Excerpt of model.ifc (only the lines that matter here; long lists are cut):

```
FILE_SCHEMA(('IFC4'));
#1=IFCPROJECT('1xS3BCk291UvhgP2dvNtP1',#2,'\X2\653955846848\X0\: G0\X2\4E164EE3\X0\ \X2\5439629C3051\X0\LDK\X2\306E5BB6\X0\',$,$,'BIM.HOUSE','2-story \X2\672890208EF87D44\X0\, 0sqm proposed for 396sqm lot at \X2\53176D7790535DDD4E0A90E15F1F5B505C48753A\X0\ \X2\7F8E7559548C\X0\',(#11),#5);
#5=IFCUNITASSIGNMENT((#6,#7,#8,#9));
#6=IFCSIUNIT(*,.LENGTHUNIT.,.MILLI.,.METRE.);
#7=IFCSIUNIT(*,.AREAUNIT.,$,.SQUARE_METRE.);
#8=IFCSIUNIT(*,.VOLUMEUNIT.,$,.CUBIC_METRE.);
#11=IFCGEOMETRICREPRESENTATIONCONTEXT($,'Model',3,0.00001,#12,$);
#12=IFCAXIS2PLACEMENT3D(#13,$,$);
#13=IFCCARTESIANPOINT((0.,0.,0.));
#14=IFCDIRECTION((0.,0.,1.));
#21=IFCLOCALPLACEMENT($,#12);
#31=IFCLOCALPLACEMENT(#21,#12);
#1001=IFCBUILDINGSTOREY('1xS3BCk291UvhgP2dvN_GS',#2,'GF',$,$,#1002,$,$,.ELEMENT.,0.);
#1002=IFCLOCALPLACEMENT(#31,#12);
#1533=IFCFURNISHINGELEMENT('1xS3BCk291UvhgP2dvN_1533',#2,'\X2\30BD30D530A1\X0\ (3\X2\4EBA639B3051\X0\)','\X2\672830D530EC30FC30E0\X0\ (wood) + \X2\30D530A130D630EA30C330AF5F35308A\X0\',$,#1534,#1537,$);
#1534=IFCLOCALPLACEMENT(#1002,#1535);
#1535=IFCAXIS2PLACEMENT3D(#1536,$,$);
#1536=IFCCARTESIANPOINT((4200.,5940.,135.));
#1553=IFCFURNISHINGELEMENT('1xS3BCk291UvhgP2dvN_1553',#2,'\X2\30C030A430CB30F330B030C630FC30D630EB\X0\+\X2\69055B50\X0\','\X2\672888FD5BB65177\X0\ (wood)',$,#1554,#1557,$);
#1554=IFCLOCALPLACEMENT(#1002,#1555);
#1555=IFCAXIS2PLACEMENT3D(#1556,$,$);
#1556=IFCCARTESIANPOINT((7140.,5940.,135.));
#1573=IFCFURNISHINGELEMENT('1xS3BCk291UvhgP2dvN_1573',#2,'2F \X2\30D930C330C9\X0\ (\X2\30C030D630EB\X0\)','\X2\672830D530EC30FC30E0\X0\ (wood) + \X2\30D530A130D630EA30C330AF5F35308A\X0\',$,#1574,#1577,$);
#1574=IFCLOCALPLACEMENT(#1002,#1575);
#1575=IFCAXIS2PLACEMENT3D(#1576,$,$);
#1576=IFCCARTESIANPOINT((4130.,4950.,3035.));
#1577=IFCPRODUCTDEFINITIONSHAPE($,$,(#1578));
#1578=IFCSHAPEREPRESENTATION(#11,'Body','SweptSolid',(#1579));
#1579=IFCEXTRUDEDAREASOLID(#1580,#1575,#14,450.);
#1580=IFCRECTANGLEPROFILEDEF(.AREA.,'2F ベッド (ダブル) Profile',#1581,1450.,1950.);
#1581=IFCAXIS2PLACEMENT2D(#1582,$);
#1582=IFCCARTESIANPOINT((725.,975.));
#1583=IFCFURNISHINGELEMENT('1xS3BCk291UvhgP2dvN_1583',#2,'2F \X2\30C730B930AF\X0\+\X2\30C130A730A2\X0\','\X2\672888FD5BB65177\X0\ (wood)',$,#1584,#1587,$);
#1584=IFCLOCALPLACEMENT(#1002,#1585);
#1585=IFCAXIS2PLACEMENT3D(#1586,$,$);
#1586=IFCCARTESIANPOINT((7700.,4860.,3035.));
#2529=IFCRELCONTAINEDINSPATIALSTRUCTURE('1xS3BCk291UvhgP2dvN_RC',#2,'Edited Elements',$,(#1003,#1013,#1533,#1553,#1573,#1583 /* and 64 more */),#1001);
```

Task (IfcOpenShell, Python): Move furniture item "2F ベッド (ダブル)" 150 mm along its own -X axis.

```python
import ifcopenshell
import ifcopenshell.api.geometry
import ifcopenshell.util.placement

model = ifcopenshell.open("model.ifc")

item = model.by_guid("1xS3BCk291UvhgP2dvN_1573")
matrix = ifcopenshell.util.placement.get_local_placement(item.ObjectPlacement)
matrix[:3, 3] -= matrix[:3, 0] * 150.0
ifcopenshell.api.geometry.edit_object_placement(model, product=item, matrix=matrix, is_si=False)

print(ifcopenshell.util.placement.get_local_placement(item.ObjectPlacement).round(3) + 0.0)

model.write("model_updated.ifc")
```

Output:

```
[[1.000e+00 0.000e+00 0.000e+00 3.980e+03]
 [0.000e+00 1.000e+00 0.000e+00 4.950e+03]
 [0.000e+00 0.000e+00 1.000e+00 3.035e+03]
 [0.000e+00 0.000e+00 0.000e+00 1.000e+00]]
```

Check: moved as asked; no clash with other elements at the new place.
